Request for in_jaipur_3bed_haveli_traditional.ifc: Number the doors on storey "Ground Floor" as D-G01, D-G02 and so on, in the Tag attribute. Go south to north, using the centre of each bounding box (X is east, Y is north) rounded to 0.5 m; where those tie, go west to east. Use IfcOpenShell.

First a look at what the model holds.

```python
import ifcopenshell
import ifcopenshell.util.element
import ifcopenshell.util.placement

model = ifcopenshell.open("in_jaipur_3bed_haveli_traditional.ifc")
print(model.schema)
storey = next(s for s in model.by_type("IfcBuildingStorey") if s.Name == "Ground Floor")
doors = [e for e in ifcopenshell.util.element.get_decomposition(storey) if e.is_a("IfcDoor")]
for e in sorted(doors, key=lambda e: e.id()):
    origin = ifcopenshell.util.placement.get_local_placement(e.ObjectPlacement)[:3, 3]
    print(e.id(), e.Tag, e.Name, origin.round(2) + 0.0, sep=" | ")
```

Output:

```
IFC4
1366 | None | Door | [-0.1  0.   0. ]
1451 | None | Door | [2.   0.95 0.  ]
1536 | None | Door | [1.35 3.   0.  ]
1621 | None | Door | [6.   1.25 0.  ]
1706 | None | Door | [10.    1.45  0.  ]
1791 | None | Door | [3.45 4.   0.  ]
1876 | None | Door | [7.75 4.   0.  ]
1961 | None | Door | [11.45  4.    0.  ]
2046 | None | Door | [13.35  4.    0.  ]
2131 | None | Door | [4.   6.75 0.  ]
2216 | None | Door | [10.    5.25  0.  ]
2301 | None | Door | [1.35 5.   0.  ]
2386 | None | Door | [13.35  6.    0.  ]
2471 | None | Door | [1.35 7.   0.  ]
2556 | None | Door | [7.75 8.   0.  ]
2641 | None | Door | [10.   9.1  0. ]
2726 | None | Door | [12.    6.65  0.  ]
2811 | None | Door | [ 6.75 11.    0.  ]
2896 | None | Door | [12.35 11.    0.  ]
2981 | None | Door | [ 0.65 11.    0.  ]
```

```python
import ifcopenshell
import ifcopenshell.geom
import ifcopenshell.util.element
import ifcopenshell.util.shape

model = ifcopenshell.open("in_jaipur_3bed_haveli_traditional.ifc")
settings = ifcopenshell.geom.settings()
settings.set("use-world-coords", True)


def centre(element):
    shape = ifcopenshell.geom.create_shape(settings, element)
    return ifcopenshell.util.shape.get_bbox_centroid(shape.geometry)


storey = next(s for s in model.by_type("IfcBuildingStorey") if s.Name == "Ground Floor")
doors = [e for e in ifcopenshell.util.element.get_decomposition(storey) if e.is_a("IfcDoor")]

# Insertion points can sit at a corner or the storey origin, so sort by the geometry (in metres).
centres = {e: centre(e) for e in doors}
doors.sort(key=lambda e: (round(centres[e][1] / 0.5), centres[e][0]))

for i, e in enumerate(doors, start=1):
    number = f"D-G{i:02d}"
    e.Tag = number
    print(e.id(), number)

model.write("in_jaipur_3bed_haveli_traditional-out.ifc")
```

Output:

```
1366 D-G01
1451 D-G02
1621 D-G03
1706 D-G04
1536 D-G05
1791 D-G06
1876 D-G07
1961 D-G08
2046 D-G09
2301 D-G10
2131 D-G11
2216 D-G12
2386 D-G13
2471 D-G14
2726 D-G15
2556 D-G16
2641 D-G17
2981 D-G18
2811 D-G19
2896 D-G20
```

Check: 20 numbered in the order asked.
